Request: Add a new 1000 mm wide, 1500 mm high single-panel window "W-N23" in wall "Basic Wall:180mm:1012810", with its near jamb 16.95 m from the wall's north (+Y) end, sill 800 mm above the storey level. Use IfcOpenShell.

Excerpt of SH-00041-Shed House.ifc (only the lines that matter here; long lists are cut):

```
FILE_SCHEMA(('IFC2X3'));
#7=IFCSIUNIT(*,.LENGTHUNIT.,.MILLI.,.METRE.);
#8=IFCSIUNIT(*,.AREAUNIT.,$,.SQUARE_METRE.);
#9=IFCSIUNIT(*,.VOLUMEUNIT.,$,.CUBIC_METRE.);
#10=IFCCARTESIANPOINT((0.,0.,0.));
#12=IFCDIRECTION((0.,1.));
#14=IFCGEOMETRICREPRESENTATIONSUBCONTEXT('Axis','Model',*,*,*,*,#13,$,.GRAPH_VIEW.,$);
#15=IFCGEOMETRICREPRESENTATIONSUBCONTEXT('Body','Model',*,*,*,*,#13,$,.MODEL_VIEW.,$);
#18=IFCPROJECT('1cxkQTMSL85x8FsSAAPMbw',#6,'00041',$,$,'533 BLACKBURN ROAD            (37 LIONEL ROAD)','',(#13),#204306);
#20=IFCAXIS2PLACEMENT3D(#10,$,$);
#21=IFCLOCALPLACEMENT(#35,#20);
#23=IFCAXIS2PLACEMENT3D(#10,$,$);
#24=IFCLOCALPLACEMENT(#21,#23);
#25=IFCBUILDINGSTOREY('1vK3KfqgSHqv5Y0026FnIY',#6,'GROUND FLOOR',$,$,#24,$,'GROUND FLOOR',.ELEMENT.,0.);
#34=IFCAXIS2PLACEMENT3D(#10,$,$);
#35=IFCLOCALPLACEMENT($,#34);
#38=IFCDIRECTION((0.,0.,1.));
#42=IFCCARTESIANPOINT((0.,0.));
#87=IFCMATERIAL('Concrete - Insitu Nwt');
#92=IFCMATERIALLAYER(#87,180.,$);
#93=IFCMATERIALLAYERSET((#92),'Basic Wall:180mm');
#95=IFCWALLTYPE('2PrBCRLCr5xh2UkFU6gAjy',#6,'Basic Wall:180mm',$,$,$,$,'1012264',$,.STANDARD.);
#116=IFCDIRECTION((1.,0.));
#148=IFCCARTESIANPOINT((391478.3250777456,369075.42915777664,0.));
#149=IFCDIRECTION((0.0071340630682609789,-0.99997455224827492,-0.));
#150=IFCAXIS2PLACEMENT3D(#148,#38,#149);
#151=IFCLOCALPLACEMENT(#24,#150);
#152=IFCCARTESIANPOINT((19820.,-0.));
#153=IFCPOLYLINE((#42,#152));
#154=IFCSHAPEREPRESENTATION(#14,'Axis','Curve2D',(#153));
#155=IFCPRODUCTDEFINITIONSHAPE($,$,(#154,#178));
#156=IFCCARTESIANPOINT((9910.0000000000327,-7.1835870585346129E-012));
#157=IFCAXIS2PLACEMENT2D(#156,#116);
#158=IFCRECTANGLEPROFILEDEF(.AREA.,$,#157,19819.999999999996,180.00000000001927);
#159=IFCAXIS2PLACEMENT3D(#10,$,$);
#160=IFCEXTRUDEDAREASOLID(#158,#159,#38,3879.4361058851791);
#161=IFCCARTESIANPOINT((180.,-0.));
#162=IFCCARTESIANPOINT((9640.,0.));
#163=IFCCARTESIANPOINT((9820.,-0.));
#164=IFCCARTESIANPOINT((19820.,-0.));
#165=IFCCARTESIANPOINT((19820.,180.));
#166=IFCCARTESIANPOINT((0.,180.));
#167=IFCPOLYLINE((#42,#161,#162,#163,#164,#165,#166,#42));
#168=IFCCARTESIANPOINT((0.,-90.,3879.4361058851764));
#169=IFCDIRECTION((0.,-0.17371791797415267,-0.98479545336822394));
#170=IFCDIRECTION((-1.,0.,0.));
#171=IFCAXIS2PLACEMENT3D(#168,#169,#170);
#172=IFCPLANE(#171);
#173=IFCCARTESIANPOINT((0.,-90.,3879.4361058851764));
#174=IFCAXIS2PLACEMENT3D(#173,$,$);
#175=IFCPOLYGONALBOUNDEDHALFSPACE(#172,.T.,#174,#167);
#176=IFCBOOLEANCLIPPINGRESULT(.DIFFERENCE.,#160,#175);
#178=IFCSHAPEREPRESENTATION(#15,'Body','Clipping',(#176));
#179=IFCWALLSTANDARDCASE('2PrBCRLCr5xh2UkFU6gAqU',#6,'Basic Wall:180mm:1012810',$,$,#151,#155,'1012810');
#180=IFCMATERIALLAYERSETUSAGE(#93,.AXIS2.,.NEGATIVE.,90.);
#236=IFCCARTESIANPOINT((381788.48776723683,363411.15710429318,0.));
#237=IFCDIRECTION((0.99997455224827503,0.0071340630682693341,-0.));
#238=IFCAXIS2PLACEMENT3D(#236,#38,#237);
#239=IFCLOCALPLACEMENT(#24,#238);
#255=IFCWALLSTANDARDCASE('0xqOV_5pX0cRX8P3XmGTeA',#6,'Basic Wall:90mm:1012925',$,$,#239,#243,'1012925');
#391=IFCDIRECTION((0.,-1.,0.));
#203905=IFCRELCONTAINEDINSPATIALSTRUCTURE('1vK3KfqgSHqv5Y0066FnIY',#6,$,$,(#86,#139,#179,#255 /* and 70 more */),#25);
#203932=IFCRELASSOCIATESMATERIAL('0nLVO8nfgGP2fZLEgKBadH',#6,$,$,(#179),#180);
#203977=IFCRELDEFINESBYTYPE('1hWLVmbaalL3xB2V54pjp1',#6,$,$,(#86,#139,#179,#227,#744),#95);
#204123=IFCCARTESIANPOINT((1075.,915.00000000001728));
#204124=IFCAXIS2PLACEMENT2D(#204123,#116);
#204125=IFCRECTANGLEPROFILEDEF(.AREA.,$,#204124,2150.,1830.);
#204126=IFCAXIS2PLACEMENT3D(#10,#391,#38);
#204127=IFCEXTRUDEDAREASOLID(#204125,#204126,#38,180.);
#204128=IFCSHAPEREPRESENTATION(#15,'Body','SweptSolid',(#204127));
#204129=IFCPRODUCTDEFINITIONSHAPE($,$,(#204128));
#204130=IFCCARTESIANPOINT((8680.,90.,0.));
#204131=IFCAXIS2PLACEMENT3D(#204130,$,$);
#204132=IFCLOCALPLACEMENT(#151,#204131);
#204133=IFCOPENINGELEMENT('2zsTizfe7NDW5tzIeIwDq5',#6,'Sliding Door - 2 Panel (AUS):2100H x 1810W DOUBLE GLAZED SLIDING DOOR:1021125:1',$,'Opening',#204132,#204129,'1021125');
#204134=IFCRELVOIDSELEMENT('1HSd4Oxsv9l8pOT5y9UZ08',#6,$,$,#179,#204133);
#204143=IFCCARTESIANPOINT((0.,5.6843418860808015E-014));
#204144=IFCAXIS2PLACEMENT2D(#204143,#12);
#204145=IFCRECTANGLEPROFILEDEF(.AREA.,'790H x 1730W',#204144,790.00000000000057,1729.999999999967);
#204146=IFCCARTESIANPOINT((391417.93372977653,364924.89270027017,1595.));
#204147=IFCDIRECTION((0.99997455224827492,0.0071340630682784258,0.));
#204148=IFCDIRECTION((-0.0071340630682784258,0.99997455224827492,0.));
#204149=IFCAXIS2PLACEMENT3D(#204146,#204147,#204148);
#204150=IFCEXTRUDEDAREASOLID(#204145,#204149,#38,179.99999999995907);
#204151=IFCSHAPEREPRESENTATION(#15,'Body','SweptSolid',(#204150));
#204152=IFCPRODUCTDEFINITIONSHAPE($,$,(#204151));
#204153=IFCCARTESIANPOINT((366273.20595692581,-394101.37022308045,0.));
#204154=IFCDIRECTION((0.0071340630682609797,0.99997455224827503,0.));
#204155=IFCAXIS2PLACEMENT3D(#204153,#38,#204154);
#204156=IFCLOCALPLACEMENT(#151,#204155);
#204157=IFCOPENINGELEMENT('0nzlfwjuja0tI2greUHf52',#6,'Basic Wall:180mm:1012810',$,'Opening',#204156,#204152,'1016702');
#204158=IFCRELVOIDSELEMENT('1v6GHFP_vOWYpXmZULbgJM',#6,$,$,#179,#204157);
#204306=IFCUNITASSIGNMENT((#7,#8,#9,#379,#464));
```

```python
import numpy as np
import ifcopenshell
import ifcopenshell.api.feature
import ifcopenshell.api.geometry
import ifcopenshell.api.root
import ifcopenshell.api.spatial
import ifcopenshell.api.type
import ifcopenshell.geom
import ifcopenshell.util.element
import ifcopenshell.util.placement
import ifcopenshell.util.representation
import ifcopenshell.util.shape
import ifcopenshell.util.unit

model = ifcopenshell.open("SH-00041-Shed House.ifc")
unit_scale = ifcopenshell.util.unit.calculate_unit_scale(model)
settings = ifcopenshell.geom.settings()


def volume(element):
    """Net volume in cubic metres, openings subtracted."""
    shape = ifcopenshell.geom.create_shape(settings, element)
    return ifcopenshell.util.shape.get_volume(shape.geometry)


wall = model.by_id(179)
storey = ifcopenshell.util.element.get_container(wall, ifc_class="IfcBuildingStorey")
context = ifcopenshell.util.representation.get_context(model, "Model", "Body", "MODEL_VIEW")
before = volume(wall)

width, height, from_end, sill = 1, 1.5, 16.95, 0.8  # metres

# The wall runs along its own X axis, and the end named is its -X end.
wall_shape = ifcopenshell.geom.create_shape(settings, wall)
x, y, z = ifcopenshell.util.shape.get_vertices(wall_shape.geometry).T
start = x.min() + from_end
face, thickness = float(y.min()), float(y.max() - y.min())
wall_matrix = ifcopenshell.util.placement.get_local_placement(wall.ObjectPlacement)
level = ifcopenshell.util.placement.get_local_placement(storey.ObjectPlacement)[2, 3]


def in_wall(x, y):
    """Placement at x, y metres in the wall's axes, at sill height."""
    matrix = wall_matrix.copy()
    matrix[:, 3] = wall_matrix @ np.array([x / unit_scale, y / unit_scale, 0.0, 1.0])
    matrix[2, 3] = level + sill / unit_scale
    return matrix


# Opening: a box that overshoots both wall faces by 50 mm.
opening = ifcopenshell.api.root.create_entity(model, ifc_class="IfcOpeningElement")
box = ifcopenshell.api.geometry.add_wall_representation(
    model, context=context, length=width, height=height, thickness=thickness + 0.1
)
ifcopenshell.api.geometry.assign_representation(model, product=opening, representation=box)
ifcopenshell.api.geometry.edit_object_placement(model, product=opening, matrix=in_wall(start, face - 0.05), is_si=False)
ifcopenshell.api.feature.add_feature(model, feature=opening, element=wall)

window = ifcopenshell.api.root.create_entity(model, ifc_class="IfcWindow", name="W-N23")
window.OverallWidth, window.OverallHeight = width / unit_scale, height / unit_scale
body = ifcopenshell.api.geometry.add_window_representation(
    model,
    context=context,
    overall_width=window.OverallWidth,
    overall_height=window.OverallHeight,
    partition_type="SINGLE_PANEL",
)
ifcopenshell.api.geometry.assign_representation(model, product=window, representation=body)
ifcopenshell.api.spatial.assign_container(model, products=[window], relating_structure=storey)
fills = ifcopenshell.api.feature.add_filling(model, opening=opening, element=window)
fills.OwnerHistory = window.OwnerHistory  # required in IFC2X3

# IFC2X3 keeps the operation on the window style.
style = ifcopenshell.api.root.create_entity(model, ifc_class="IfcWindowStyle", name="W-N23")
style.OperationType, style.ConstructionType = "SINGLE_PANEL", "NOTDEFINED"
style.ParameterTakesPrecedence = style.Sizeable = False
ifcopenshell.api.type.assign_type(model, related_objects=[window], relating_type=style)

# Centre the window in the wall's thickness.
ifcopenshell.api.geometry.edit_object_placement(model, product=window, matrix=in_wall(start, face), is_si=False)
window_shape = ifcopenshell.geom.create_shape(settings, window)
depth = ifcopenshell.util.shape.get_vertices(window_shape.geometry)[:, 1]
offset = face + thickness / 2 - (depth.min() + depth.max()) / 2
ifcopenshell.api.geometry.edit_object_placement(model, product=window, matrix=in_wall(start, offset), is_si=False)

after = volume(wall)

print(f"wall volume {before:.3f} -> {after:.3f} m3")

model.write("SH-00041-Shed House_updated.ifc")
```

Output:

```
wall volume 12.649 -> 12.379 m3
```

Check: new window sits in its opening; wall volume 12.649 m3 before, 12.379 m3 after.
